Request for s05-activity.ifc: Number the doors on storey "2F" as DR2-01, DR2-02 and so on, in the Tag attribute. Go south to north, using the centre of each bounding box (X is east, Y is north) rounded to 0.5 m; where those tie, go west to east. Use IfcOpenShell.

First a look at what the model holds.

```python
import ifcopenshell
import ifcopenshell.util.element
import ifcopenshell.util.placement

model = ifcopenshell.open("s05-activity.ifc")
print(model.schema)
storey = next(s for s in model.by_type("IfcBuildingStorey") if s.Name == "2F")
doors = [e for e in ifcopenshell.util.element.get_decomposition(storey) if e.is_a("IfcDoor")]
for e in sorted(doors, key=lambda e: e.id()):
    origin = ifcopenshell.util.placement.get_local_placement(e.ObjectPlacement)[:3, 3]
    print(e.id(), e.Tag, e.Name, origin.round(2) + 0.0, sep=" | ")
```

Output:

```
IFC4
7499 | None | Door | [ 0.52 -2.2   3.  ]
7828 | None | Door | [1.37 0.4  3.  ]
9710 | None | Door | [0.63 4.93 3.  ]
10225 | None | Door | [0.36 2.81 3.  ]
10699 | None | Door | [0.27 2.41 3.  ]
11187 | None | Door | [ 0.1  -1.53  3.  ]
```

```python
import ifcopenshell
import ifcopenshell.geom
import ifcopenshell.util.element
import ifcopenshell.util.shape

model = ifcopenshell.open("s05-activity.ifc")
settings = ifcopenshell.geom.settings()
settings.set("use-world-coords", True)


def centre(element):
    shape = ifcopenshell.geom.create_shape(settings, element)
    return ifcopenshell.util.shape.get_bbox_centroid(shape.geometry)


storey = next(s for s in model.by_type("IfcBuildingStorey") if s.Name == "2F")
doors = [e for e in ifcopenshell.util.element.get_decomposition(storey) if e.is_a("IfcDoor")]

# Insertion points can sit at a corner or the storey origin, so sort by the geometry (in metres).
centres = {e: centre(e) for e in doors}
doors.sort(key=lambda e: (round(centres[e][1] / 0.5), centres[e][0]))

for i, e in enumerate(doors, start=1):
    number = f"DR2-{i:02d}"
    e.Tag = number
    print(e.id(), number)

model.write("s05-activity-out.ifc")
```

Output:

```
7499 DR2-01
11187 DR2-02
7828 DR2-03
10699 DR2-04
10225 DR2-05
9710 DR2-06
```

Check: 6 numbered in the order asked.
